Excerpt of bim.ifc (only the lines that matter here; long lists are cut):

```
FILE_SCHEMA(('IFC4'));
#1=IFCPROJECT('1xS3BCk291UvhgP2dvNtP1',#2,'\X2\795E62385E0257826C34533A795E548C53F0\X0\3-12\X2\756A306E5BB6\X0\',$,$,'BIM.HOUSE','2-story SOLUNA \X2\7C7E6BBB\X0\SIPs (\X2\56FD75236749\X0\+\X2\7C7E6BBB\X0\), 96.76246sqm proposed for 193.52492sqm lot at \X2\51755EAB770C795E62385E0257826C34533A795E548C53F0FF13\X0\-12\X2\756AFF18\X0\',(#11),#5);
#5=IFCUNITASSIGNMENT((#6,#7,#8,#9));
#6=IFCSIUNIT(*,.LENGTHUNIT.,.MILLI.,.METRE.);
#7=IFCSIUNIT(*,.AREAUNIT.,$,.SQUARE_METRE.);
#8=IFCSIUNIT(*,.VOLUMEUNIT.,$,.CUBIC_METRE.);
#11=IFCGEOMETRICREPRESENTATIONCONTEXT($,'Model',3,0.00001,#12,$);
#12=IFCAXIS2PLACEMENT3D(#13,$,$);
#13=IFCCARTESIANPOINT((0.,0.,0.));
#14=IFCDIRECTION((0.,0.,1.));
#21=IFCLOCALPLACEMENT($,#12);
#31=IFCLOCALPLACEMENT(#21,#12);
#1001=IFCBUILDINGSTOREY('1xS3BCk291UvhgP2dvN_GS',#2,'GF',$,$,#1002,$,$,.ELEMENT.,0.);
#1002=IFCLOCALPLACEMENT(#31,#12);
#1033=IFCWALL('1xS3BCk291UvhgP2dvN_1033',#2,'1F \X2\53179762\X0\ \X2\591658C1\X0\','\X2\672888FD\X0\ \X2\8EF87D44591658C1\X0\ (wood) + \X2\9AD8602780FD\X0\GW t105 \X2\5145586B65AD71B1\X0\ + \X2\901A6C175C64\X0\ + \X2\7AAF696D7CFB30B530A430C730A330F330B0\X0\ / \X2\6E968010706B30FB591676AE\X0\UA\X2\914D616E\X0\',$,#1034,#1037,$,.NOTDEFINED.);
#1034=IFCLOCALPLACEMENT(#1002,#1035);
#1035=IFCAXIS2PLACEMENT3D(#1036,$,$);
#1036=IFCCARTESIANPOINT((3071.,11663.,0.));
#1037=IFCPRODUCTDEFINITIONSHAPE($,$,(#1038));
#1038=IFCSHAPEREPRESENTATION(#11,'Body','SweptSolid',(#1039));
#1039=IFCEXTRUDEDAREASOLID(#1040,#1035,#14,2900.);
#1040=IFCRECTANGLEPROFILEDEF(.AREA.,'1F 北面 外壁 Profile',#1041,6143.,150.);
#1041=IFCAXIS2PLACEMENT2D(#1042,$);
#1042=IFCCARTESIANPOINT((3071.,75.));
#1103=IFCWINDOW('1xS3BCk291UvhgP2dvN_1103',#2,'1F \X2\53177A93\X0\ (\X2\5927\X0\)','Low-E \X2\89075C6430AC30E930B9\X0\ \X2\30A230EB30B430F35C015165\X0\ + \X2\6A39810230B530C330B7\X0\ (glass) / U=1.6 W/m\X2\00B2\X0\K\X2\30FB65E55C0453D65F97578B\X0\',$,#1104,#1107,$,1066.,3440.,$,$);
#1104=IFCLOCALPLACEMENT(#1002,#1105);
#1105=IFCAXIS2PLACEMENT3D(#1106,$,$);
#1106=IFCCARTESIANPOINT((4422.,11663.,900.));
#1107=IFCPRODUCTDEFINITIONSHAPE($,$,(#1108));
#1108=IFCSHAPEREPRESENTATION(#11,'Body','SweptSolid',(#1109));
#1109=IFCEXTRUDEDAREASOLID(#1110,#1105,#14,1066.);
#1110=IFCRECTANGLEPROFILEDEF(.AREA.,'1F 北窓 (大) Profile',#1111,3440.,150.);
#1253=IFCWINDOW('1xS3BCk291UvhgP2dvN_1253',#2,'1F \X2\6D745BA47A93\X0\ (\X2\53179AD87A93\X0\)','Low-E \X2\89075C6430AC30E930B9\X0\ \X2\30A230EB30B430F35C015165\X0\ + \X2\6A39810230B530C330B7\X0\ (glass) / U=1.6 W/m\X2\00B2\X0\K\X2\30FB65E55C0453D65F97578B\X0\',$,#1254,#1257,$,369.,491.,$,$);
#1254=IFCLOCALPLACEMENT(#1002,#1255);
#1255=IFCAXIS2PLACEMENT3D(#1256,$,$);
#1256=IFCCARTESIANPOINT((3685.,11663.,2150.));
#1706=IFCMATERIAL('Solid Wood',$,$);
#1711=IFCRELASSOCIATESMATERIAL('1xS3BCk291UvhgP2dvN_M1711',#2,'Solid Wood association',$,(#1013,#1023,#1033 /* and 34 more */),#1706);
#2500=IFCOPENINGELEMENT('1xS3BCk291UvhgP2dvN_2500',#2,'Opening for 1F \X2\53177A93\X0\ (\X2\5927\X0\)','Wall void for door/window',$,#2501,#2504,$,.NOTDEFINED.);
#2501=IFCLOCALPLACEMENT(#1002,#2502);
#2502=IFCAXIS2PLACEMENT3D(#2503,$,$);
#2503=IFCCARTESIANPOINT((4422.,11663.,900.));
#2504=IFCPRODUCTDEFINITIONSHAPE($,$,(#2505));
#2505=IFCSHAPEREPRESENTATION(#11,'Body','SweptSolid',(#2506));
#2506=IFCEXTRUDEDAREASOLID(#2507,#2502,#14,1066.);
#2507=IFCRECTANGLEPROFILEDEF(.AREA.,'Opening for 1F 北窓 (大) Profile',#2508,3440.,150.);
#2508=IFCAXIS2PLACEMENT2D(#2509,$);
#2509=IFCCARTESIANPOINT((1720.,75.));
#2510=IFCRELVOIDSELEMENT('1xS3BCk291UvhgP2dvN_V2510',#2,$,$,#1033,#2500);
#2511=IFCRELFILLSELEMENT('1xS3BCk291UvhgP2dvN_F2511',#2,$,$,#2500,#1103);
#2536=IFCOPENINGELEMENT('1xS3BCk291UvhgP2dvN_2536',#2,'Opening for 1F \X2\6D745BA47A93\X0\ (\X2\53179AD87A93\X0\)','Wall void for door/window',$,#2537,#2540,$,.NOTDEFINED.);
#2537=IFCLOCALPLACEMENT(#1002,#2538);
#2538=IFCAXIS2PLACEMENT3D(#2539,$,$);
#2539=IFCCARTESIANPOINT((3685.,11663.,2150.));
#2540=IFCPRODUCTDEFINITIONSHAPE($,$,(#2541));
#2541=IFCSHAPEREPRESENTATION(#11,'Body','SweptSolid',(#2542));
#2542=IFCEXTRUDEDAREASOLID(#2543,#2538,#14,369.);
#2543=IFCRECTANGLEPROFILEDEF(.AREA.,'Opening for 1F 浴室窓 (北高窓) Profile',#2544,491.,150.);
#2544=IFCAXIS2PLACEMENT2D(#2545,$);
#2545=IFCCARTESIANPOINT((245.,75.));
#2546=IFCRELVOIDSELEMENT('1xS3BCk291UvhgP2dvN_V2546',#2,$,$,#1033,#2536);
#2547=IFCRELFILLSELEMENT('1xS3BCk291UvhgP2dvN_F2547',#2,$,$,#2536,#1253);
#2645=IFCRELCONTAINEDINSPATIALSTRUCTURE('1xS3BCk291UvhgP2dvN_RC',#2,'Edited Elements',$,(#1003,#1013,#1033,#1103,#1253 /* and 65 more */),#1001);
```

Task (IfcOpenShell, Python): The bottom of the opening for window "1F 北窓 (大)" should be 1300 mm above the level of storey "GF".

```python
import numpy as np
import ifcopenshell
import ifcopenshell.api.geometry
import ifcopenshell.geom
import ifcopenshell.util.element
import ifcopenshell.util.placement
import ifcopenshell.util.shape
import ifcopenshell.util.unit

model = ifcopenshell.open("bim.ifc")
unit_scale = ifcopenshell.util.unit.calculate_unit_scale(model)

window = model.by_guid("1xS3BCk291UvhgP2dvN_1103")
opening = window.FillsVoids[0].RelatingOpeningElement
storey = ifcopenshell.util.element.get_container(window, ifc_class="IfcBuildingStorey")
level = ifcopenshell.util.placement.get_local_placement(storey.ObjectPlacement)[2, 3]

# The opening's origin need not be at the sill, so measure its lowest point.
shape = ifcopenshell.geom.create_shape(ifcopenshell.geom.settings(), opening)
bottom = ifcopenshell.util.shape.get_shape_bottom_elevation(shape, shape.geometry) / unit_scale
dz = level + 1300.0 - bottom

shift = np.array([0.0, 0.0, dz])
# The window is not placed relative to its opening, so move both.
for product in (opening, window):
    matrix = ifcopenshell.util.placement.get_local_placement(product.ObjectPlacement)
    matrix[:3, 3] += shift
    ifcopenshell.api.geometry.edit_object_placement(model, product=product, matrix=matrix, is_si=False)

print(f"moved by {dz * unit_scale:+.3f} m")

model.write("bim-out.ifc")
```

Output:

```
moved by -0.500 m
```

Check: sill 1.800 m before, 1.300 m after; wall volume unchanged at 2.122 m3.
